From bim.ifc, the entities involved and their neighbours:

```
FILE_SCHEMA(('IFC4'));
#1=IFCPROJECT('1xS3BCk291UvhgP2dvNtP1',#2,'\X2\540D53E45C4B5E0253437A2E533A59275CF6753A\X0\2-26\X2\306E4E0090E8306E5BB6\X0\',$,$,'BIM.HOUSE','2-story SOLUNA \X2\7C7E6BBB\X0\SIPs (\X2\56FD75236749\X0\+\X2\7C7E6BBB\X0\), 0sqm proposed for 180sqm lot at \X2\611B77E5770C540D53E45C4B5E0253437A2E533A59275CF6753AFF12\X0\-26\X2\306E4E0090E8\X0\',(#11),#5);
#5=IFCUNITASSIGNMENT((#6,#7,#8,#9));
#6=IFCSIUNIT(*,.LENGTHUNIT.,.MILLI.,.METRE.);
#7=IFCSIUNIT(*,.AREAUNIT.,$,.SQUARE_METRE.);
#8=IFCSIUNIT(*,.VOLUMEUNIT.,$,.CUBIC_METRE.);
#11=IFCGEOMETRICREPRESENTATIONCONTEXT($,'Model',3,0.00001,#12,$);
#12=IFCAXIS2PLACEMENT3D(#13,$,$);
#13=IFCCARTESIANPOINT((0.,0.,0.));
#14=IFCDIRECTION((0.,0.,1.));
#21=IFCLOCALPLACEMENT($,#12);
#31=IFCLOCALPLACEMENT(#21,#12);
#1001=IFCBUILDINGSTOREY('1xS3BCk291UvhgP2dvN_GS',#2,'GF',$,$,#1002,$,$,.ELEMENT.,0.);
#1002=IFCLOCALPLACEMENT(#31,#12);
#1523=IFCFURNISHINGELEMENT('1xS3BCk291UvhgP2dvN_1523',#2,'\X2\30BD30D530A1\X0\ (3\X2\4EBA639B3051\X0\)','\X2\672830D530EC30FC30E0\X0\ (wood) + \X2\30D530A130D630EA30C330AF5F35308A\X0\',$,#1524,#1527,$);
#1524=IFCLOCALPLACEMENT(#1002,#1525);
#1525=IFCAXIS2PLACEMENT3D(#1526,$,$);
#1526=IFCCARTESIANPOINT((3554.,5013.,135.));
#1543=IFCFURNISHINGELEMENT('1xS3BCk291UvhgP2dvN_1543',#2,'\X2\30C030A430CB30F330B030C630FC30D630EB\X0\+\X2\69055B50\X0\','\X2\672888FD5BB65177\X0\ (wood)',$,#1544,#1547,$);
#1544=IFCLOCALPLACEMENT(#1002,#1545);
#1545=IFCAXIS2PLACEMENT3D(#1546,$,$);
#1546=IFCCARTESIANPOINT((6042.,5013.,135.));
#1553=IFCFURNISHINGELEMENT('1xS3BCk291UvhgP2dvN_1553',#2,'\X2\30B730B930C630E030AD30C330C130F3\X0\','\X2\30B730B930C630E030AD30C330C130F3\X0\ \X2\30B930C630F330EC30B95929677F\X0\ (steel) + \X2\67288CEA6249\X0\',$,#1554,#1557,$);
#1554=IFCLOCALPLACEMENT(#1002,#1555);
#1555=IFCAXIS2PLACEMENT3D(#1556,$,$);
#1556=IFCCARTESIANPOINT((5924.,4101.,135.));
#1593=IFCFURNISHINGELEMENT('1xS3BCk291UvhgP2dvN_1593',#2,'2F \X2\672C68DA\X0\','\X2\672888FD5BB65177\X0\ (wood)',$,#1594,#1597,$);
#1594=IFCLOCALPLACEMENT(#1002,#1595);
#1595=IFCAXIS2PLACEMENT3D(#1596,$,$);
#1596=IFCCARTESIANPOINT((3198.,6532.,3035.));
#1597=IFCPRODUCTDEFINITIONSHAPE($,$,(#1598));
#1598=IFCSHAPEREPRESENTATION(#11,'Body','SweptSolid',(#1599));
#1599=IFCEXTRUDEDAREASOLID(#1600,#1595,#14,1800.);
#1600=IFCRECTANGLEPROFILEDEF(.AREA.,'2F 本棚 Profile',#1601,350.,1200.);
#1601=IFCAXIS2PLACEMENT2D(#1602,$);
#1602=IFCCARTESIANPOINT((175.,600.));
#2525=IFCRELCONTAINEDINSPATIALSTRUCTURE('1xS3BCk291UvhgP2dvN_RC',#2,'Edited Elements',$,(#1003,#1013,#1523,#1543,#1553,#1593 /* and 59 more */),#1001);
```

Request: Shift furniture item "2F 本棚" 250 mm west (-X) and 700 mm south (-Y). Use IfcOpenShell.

```python
import ifcopenshell
import ifcopenshell.api.geometry
import ifcopenshell.util.placement
import ifcopenshell.util.unit

model = ifcopenshell.open("bim.ifc")
unit_scale = ifcopenshell.util.unit.calculate_unit_scale(model)

item = model.by_guid("1xS3BCk291UvhgP2dvN_1593")
matrix = ifcopenshell.util.placement.get_local_placement(item.ObjectPlacement)
matrix[0, 3] -= 0.25 / unit_scale
matrix[1, 3] -= 0.7 / unit_scale
ifcopenshell.api.geometry.edit_object_placement(model, product=item, matrix=matrix, is_si=False)

print(ifcopenshell.util.placement.get_local_placement(item.ObjectPlacement).round(3) + 0.0)

model.write("bim_v2.ifc")
```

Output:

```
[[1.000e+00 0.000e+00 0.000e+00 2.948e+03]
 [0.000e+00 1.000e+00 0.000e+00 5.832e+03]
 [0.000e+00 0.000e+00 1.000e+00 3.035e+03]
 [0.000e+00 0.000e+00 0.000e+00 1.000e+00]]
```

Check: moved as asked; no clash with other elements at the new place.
